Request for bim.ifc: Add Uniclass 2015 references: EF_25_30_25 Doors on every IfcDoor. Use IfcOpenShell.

First a look at what the model holds.

```python
import ifcopenshell

model = ifcopenshell.open("bim.ifc")
print(model.schema)
print("classifications:", [c.Name for c in model.by_type("IfcClassification")])
for ifc_class in ("IfcDoor", "IfcRoof", "IfcStair", "IfcWall", "IfcWindow"):
    print(ifc_class, len(model.by_type(ifc_class)))
```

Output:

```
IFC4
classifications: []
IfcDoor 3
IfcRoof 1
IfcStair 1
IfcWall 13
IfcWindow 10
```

```python
import ifcopenshell
import ifcopenshell.api.classification

model = ifcopenshell.open("bim.ifc")

system = ifcopenshell.api.classification.add_classification(model, classification="Uniclass 2015")

codes = {
    "IfcDoor": ("EF_25_30_25", "Doors"),
}
for ifc_class, (code, name) in codes.items():
    products = model.by_type(ifc_class)
    ifcopenshell.api.classification.add_reference(
        model, products=products, classification=system, identification=code, name=name
    )
    print(code, len(products))

model.write("bim_v2.ifc")
```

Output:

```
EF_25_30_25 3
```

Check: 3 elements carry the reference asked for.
